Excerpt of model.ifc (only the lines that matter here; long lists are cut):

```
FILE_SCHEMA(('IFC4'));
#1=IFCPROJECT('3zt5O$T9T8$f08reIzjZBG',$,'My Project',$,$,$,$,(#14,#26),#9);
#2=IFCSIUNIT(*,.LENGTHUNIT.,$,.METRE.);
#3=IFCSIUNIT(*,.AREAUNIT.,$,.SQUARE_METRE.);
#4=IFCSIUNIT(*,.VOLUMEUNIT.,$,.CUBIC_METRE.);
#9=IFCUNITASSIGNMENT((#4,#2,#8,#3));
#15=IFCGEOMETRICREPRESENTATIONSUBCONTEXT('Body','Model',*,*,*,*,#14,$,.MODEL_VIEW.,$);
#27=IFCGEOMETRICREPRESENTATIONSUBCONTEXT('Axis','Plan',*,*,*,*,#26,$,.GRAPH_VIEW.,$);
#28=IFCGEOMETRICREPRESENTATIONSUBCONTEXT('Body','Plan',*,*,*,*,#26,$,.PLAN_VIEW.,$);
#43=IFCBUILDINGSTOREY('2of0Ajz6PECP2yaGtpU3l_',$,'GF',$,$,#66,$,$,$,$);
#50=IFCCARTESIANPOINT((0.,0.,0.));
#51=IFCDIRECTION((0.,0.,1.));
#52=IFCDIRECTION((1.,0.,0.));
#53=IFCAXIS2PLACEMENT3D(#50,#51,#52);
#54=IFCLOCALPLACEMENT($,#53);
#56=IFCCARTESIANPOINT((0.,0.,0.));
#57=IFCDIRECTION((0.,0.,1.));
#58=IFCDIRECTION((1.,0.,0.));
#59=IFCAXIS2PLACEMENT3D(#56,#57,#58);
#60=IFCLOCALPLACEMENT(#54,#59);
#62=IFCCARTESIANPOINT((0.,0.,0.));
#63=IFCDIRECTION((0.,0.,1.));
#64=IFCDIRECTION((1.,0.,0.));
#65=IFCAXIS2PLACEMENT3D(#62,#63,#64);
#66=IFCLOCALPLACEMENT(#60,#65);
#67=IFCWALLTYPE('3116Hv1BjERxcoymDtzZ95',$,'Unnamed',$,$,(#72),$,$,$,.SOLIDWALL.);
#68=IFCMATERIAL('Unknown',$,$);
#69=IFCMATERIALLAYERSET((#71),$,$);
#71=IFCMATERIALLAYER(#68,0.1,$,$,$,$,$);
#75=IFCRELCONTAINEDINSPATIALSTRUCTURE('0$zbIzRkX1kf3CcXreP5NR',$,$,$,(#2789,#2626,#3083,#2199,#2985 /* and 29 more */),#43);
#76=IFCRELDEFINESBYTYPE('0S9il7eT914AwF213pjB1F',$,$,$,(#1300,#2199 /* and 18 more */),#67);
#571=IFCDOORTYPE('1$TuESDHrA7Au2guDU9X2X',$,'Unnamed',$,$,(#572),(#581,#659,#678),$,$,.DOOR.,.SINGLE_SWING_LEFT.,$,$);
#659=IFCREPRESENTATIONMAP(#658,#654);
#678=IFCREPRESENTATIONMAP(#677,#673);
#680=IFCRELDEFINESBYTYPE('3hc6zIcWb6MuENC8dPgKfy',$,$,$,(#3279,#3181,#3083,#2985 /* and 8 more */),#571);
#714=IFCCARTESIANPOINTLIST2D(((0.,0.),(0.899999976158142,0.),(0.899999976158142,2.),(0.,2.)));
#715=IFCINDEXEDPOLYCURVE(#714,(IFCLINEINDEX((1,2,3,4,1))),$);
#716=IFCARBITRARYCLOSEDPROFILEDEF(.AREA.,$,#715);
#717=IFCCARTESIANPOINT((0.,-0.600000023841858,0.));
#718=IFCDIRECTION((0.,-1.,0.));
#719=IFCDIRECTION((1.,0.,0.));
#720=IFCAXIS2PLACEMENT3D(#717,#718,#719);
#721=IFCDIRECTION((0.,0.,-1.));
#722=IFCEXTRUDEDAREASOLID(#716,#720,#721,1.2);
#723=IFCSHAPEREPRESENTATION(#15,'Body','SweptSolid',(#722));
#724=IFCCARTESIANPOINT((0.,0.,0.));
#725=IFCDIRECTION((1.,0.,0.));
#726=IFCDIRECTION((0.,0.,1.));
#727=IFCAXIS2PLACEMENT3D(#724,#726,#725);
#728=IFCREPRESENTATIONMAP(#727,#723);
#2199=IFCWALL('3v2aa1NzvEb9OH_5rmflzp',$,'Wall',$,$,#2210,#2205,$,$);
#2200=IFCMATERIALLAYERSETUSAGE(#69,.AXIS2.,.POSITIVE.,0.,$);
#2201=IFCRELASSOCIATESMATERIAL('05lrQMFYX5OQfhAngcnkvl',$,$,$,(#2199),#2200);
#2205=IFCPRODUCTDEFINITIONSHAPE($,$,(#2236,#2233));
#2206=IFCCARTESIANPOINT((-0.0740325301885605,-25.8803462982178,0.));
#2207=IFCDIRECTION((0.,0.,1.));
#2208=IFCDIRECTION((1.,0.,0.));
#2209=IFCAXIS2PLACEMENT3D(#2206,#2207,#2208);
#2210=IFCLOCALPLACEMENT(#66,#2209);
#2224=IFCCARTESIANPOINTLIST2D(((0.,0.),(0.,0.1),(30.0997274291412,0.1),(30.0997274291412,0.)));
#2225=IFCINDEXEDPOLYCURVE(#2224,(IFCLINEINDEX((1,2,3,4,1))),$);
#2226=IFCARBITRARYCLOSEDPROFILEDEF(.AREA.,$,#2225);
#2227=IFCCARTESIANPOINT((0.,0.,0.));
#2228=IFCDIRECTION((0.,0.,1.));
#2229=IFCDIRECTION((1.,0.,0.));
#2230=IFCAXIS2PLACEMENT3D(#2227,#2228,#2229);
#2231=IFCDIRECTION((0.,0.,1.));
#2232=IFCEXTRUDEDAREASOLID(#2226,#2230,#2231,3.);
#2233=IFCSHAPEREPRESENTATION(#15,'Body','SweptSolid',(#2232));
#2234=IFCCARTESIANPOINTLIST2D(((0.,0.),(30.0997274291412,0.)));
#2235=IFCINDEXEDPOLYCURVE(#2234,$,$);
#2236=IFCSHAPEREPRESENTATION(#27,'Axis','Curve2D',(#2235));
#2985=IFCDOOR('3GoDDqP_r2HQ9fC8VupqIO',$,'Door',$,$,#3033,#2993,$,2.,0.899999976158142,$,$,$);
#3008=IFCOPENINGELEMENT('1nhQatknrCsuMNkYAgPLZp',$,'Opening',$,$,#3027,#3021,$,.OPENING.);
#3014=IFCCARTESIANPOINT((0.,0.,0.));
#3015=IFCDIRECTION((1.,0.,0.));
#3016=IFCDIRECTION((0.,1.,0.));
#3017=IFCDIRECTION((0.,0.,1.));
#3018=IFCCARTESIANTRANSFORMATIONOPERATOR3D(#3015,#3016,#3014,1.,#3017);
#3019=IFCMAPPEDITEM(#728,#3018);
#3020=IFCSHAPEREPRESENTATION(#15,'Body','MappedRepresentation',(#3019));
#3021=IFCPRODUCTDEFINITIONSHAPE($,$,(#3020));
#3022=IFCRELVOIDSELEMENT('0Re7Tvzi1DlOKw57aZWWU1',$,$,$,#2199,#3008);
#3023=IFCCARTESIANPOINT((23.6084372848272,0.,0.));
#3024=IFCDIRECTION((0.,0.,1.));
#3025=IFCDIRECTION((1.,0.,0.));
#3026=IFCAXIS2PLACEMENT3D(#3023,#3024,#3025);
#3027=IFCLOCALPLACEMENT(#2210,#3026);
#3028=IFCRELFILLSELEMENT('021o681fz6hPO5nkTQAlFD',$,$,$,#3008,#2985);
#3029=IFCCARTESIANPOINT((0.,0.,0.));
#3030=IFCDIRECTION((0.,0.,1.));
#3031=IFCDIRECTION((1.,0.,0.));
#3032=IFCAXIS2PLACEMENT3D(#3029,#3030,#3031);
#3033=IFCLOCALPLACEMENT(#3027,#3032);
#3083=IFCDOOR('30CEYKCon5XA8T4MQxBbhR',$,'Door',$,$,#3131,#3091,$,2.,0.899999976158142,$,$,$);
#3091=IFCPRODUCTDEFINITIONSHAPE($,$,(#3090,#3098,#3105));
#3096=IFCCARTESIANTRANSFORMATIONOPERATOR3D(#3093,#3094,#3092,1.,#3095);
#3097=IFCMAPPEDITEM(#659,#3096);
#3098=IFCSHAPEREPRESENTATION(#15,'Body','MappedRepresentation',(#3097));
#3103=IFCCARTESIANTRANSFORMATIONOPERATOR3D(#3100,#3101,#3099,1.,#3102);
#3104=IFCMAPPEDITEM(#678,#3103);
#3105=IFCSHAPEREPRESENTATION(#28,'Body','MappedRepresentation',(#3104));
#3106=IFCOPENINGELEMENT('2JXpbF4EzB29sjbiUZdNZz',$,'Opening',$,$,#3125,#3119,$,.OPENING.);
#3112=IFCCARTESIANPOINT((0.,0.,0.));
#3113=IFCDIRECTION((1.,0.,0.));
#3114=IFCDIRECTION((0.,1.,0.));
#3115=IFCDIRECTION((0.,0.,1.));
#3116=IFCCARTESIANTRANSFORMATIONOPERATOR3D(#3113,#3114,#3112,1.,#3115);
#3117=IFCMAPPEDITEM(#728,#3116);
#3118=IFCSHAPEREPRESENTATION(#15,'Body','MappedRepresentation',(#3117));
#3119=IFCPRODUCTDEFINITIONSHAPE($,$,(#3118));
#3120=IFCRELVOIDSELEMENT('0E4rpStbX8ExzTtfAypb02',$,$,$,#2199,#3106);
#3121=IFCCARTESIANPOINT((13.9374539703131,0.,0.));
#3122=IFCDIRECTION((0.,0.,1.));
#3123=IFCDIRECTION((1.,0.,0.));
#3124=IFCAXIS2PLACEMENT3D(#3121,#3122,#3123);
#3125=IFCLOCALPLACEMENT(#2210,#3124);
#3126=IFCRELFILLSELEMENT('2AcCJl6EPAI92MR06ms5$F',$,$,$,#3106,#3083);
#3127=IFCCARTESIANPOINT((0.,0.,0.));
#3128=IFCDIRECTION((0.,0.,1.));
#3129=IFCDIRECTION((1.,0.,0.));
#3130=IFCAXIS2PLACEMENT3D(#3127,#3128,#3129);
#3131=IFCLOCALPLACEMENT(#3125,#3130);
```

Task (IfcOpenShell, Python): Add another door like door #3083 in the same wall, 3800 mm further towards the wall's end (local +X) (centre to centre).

```python
import ifcopenshell
import ifcopenshell.api.feature
import ifcopenshell.api.geometry
import ifcopenshell.api.root
import ifcopenshell.geom
import ifcopenshell.util.element
import ifcopenshell.util.placement
import ifcopenshell.util.shape
import ifcopenshell.util.unit

model = ifcopenshell.open("model.ifc")
unit_scale = ifcopenshell.util.unit.calculate_unit_scale(model)
settings = ifcopenshell.geom.settings()


def volume(element):
    """Net volume in cubic metres, openings subtracted."""
    shape = ifcopenshell.geom.create_shape(settings, element)
    return ifcopenshell.util.shape.get_volume(shape.geometry)


door = model.by_guid("30CEYKCon5XA8T4MQxBbhR")
opening = door.FillsVoids[0].RelatingOpeningElement
wall = opening.VoidsElements[0].RelatingBuildingElement
before = volume(wall)
shift = ifcopenshell.util.placement.get_local_placement(wall.ObjectPlacement)[:3, 0] * 3.8 / unit_scale

# copy_class copies the void relationship, type, container and properties, but no geometry.
new_opening = ifcopenshell.api.root.copy_class(model, product=opening)
new_opening.Representation = ifcopenshell.util.element.copy_deep(
    model, opening.Representation, exclude=["IfcGeometricRepresentationContext", "IfcRepresentationMap"]
)
new_door = ifcopenshell.api.root.copy_class(model, product=door)
new_door.Representation = ifcopenshell.util.element.copy_deep(
    model, door.Representation, exclude=["IfcGeometricRepresentationContext", "IfcRepresentationMap"]
)
ifcopenshell.api.feature.add_filling(model, opening=new_opening, element=new_door)

for old, new in ((opening, new_opening), (door, new_door)):
    matrix = ifcopenshell.util.placement.get_local_placement(old.ObjectPlacement)
    matrix[:3, 3] += shift
    ifcopenshell.api.geometry.edit_object_placement(model, product=new, matrix=matrix, is_si=False)

after = volume(wall)

print(f"wall volume {before:.3f} -> {after:.3f} m3")

model.write("model_v2.ifc")
```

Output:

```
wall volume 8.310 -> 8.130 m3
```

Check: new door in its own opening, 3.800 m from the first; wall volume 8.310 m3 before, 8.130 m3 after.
